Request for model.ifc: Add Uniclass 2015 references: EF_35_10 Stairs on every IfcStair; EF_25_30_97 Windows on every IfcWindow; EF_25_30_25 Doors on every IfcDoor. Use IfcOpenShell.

First a look at what the model holds.

```python
import ifcopenshell

model = ifcopenshell.open("model.ifc")
print(model.schema)
print("classifications:", [c.Name for c in model.by_type("IfcClassification")])
for ifc_class in ("IfcDoor", "IfcRoof", "IfcStair", "IfcWall", "IfcWindow"):
    print(ifc_class, len(model.by_type(ifc_class)))
```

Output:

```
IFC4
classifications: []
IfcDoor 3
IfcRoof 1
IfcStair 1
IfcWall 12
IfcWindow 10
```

```python
import ifcopenshell
import ifcopenshell.api.classification

model = ifcopenshell.open("model.ifc")

system = ifcopenshell.api.classification.add_classification(model, classification="Uniclass 2015")

codes = {
    "IfcStair": ("EF_35_10", "Stairs"),
    "IfcWindow": ("EF_25_30_97", "Windows"),
    "IfcDoor": ("EF_25_30_25", "Doors"),
}
for ifc_class, (code, name) in codes.items():
    products = model.by_type(ifc_class)
    ifcopenshell.api.classification.add_reference(
        model, products=products, classification=system, identification=code, name=name
    )
    print(code, len(products))

model.write("model_updated.ifc")
```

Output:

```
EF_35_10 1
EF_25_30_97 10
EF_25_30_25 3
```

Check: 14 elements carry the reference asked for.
